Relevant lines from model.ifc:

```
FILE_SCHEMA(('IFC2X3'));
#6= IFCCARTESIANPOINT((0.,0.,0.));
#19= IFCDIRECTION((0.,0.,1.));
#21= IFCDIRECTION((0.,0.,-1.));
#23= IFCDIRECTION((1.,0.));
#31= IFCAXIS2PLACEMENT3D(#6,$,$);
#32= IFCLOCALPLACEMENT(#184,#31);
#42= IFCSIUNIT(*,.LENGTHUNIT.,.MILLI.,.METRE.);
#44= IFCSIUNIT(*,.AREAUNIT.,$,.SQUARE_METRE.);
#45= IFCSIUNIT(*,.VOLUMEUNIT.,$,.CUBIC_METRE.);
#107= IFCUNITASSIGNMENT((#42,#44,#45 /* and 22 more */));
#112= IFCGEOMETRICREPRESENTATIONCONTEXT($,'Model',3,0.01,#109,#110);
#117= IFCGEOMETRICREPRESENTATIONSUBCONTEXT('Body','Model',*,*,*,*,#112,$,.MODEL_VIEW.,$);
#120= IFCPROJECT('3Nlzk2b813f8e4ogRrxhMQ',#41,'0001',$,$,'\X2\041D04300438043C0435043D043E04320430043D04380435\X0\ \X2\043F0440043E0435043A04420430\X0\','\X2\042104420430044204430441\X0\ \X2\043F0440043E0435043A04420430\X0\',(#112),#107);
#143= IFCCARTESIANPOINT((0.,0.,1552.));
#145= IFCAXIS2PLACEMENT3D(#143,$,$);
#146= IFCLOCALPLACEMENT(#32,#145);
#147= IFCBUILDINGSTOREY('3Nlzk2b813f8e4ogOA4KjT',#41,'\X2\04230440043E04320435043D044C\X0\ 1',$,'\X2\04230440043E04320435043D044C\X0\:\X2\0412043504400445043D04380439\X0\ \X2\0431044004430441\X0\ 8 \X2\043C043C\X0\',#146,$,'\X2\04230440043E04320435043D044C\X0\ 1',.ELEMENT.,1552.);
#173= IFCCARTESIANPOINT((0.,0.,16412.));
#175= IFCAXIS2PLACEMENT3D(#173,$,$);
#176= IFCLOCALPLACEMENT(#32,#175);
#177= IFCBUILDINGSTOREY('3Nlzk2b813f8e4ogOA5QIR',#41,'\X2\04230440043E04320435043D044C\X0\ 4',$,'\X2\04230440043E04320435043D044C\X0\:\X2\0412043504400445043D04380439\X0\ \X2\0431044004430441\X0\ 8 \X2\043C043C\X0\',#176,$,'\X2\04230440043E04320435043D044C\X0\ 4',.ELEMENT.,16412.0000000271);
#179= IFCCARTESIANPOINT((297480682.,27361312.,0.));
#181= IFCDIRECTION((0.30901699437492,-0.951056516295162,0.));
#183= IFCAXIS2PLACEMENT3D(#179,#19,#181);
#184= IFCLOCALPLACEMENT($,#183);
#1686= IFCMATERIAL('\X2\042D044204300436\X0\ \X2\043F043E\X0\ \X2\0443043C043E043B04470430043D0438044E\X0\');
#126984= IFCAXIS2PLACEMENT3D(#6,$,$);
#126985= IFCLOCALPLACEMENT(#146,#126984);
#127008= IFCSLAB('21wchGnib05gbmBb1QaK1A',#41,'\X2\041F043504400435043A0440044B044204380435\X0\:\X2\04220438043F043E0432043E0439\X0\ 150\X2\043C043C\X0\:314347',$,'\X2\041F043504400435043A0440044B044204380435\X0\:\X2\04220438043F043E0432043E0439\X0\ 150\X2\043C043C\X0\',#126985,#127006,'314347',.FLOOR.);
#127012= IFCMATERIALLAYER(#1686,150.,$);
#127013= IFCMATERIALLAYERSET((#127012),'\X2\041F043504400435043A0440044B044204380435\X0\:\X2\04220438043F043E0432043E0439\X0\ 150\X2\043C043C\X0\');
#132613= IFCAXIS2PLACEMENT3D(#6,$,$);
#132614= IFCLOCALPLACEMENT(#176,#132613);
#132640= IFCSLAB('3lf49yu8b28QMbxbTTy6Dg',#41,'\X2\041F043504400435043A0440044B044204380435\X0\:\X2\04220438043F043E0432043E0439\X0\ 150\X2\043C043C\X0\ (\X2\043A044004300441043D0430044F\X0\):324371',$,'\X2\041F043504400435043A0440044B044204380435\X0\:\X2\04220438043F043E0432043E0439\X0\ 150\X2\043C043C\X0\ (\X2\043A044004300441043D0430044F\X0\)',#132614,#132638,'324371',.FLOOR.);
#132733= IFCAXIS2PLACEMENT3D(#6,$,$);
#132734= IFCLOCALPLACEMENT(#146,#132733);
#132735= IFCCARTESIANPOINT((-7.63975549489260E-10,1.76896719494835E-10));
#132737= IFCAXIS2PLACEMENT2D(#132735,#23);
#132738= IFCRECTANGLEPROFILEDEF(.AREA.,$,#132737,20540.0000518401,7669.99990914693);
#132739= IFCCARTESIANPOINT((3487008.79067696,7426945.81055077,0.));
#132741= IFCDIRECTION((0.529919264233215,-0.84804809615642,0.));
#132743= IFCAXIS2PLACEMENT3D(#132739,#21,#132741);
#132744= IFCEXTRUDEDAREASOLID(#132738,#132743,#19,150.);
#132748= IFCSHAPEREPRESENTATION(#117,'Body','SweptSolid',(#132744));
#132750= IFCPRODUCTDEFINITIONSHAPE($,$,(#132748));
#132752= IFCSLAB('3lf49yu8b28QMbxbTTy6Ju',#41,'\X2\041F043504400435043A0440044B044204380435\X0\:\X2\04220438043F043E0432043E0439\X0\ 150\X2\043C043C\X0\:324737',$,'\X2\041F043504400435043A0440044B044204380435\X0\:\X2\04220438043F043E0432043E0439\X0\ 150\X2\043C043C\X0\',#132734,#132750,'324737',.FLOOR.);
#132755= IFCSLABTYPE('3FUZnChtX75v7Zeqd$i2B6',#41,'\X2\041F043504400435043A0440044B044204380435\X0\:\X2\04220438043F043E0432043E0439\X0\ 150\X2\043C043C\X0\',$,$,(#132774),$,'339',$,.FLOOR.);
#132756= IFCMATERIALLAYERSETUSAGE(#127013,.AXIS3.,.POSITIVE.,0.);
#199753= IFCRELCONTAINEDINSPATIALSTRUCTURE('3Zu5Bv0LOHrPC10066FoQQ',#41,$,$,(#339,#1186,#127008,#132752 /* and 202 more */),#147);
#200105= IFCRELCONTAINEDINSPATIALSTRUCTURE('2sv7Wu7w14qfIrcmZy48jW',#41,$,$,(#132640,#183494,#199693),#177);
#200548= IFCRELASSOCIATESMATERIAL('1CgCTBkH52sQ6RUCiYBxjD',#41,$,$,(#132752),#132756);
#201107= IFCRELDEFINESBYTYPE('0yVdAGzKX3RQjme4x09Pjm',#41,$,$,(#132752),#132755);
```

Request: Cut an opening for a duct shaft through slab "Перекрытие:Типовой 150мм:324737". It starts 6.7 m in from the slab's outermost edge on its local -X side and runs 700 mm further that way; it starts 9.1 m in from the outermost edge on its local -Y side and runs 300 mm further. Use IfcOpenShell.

```python
import numpy as np
import ifcopenshell
import ifcopenshell.api.feature
import ifcopenshell.api.geometry
import ifcopenshell.api.root
import ifcopenshell.geom
import ifcopenshell.util.placement
import ifcopenshell.util.representation
import ifcopenshell.util.shape
import ifcopenshell.util.unit

model = ifcopenshell.open("model.ifc")
unit_scale = ifcopenshell.util.unit.calculate_unit_scale(model)
settings = ifcopenshell.geom.settings()


def volume(element):
    """Net volume in cubic metres, openings subtracted."""
    shape = ifcopenshell.geom.create_shape(settings, element)
    return ifcopenshell.util.shape.get_volume(shape.geometry)


slab = model.by_guid("3lf49yu8b28QMbxbTTy6Ju")
before = volume(slab)

# Extent in the slab's own axes, in metres. The edges named are its -X and -Y sides.
slab_shape = ifcopenshell.geom.create_shape(settings, slab)
vertices = ifcopenshell.util.shape.get_vertices(slab_shape.geometry)
x_min, y_min, bottom = vertices.min(axis=0)
top = vertices[:, 2].max()

opening = ifcopenshell.api.root.create_entity(model, ifc_class="IfcOpeningElement", name="Duct shaft opening")
context = ifcopenshell.util.representation.get_context(model, "Model", "Body", "MODEL_VIEW")
width, depth = 0.7, 0.3
outline = [(0.0, 0.0), (width, 0.0), (width, depth), (0.0, depth), (0.0, 0.0)]
# Overshoot both faces by 50 mm so the cut is clean.
shape = ifcopenshell.api.geometry.add_slab_representation(
    model, context=context, depth=top - bottom + 0.1, polyline=outline
)
ifcopenshell.api.geometry.assign_representation(model, product=opening, representation=shape)

matrix = ifcopenshell.util.placement.get_local_placement(slab.ObjectPlacement)
matrix[:, 3] = matrix @ np.append(np.array([x_min + 6.7, y_min + 9.1, bottom - 0.05]) / unit_scale, 1.0)
ifcopenshell.api.geometry.edit_object_placement(model, product=opening, matrix=matrix, is_si=False)
ifcopenshell.api.feature.add_feature(model, feature=opening, element=slab)

after = volume(slab)

print(f"slab volume {before:.3f} -> {after:.3f} m3")

model.write("model_v2.ifc")
```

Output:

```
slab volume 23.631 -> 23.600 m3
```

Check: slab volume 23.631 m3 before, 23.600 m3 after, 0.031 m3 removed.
